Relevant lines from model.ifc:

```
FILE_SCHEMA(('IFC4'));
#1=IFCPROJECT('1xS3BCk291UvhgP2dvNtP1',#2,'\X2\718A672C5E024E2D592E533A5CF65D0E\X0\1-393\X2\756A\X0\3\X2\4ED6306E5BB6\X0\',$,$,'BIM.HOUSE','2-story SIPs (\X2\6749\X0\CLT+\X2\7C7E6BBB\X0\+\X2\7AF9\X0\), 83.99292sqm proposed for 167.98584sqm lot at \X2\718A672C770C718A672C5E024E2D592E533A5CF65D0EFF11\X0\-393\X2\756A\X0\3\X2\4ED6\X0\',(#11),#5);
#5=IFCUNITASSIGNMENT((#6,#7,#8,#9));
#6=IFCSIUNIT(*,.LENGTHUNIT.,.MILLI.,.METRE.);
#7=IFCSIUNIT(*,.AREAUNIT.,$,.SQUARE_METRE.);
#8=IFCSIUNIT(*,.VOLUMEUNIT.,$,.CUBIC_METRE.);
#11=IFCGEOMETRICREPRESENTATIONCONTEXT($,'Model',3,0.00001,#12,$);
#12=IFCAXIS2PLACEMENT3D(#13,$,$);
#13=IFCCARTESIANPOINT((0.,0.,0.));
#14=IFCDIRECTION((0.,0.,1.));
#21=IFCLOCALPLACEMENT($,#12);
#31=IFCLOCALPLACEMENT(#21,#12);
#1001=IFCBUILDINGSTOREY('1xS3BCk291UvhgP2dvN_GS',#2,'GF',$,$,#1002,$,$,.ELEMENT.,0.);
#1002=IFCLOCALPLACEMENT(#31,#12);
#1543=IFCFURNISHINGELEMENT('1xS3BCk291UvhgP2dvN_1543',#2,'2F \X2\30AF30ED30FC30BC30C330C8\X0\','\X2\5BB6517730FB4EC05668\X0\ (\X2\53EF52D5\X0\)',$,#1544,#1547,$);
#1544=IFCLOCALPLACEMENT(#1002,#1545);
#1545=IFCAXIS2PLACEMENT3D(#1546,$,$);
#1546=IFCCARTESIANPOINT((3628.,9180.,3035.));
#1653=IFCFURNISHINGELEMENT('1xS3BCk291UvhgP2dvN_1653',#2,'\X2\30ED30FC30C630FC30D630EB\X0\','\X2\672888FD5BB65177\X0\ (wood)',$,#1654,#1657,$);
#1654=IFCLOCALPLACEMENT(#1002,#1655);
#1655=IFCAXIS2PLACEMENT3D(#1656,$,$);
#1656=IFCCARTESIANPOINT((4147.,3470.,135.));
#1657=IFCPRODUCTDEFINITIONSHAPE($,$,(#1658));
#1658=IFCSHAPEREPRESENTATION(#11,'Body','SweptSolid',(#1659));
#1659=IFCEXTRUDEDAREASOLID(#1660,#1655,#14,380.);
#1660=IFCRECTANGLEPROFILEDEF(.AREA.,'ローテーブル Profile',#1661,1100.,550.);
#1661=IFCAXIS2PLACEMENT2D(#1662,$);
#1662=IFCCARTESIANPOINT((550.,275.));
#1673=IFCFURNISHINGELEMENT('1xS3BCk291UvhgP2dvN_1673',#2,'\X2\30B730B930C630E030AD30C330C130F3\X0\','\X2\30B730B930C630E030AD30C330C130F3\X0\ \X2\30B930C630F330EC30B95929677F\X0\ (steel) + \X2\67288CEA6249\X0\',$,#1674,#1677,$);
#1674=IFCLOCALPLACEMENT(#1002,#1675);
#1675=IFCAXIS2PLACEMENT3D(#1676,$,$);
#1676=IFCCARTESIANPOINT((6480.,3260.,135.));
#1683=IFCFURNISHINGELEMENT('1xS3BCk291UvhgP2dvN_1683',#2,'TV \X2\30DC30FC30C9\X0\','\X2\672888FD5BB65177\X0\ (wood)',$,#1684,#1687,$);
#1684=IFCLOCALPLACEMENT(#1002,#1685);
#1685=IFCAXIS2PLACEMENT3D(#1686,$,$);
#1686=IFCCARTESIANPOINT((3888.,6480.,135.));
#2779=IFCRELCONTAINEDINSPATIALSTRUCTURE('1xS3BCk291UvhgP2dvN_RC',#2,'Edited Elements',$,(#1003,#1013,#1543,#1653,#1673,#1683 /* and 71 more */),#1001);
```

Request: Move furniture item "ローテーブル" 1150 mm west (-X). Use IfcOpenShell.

```python
import ifcopenshell
import ifcopenshell.api.geometry
import ifcopenshell.util.placement

model = ifcopenshell.open("model.ifc")

item = model.by_guid("1xS3BCk291UvhgP2dvN_1653")
matrix = ifcopenshell.util.placement.get_local_placement(item.ObjectPlacement)
matrix[0, 3] -= 1150.0
ifcopenshell.api.geometry.edit_object_placement(model, product=item, matrix=matrix, is_si=False)

print(ifcopenshell.util.placement.get_local_placement(item.ObjectPlacement).round(3) + 0.0)

model.write("model_rev.ifc")
```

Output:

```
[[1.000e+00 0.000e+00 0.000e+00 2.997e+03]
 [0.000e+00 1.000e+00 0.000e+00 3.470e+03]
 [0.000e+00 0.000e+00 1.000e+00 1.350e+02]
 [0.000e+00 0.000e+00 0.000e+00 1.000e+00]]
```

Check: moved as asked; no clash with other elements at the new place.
